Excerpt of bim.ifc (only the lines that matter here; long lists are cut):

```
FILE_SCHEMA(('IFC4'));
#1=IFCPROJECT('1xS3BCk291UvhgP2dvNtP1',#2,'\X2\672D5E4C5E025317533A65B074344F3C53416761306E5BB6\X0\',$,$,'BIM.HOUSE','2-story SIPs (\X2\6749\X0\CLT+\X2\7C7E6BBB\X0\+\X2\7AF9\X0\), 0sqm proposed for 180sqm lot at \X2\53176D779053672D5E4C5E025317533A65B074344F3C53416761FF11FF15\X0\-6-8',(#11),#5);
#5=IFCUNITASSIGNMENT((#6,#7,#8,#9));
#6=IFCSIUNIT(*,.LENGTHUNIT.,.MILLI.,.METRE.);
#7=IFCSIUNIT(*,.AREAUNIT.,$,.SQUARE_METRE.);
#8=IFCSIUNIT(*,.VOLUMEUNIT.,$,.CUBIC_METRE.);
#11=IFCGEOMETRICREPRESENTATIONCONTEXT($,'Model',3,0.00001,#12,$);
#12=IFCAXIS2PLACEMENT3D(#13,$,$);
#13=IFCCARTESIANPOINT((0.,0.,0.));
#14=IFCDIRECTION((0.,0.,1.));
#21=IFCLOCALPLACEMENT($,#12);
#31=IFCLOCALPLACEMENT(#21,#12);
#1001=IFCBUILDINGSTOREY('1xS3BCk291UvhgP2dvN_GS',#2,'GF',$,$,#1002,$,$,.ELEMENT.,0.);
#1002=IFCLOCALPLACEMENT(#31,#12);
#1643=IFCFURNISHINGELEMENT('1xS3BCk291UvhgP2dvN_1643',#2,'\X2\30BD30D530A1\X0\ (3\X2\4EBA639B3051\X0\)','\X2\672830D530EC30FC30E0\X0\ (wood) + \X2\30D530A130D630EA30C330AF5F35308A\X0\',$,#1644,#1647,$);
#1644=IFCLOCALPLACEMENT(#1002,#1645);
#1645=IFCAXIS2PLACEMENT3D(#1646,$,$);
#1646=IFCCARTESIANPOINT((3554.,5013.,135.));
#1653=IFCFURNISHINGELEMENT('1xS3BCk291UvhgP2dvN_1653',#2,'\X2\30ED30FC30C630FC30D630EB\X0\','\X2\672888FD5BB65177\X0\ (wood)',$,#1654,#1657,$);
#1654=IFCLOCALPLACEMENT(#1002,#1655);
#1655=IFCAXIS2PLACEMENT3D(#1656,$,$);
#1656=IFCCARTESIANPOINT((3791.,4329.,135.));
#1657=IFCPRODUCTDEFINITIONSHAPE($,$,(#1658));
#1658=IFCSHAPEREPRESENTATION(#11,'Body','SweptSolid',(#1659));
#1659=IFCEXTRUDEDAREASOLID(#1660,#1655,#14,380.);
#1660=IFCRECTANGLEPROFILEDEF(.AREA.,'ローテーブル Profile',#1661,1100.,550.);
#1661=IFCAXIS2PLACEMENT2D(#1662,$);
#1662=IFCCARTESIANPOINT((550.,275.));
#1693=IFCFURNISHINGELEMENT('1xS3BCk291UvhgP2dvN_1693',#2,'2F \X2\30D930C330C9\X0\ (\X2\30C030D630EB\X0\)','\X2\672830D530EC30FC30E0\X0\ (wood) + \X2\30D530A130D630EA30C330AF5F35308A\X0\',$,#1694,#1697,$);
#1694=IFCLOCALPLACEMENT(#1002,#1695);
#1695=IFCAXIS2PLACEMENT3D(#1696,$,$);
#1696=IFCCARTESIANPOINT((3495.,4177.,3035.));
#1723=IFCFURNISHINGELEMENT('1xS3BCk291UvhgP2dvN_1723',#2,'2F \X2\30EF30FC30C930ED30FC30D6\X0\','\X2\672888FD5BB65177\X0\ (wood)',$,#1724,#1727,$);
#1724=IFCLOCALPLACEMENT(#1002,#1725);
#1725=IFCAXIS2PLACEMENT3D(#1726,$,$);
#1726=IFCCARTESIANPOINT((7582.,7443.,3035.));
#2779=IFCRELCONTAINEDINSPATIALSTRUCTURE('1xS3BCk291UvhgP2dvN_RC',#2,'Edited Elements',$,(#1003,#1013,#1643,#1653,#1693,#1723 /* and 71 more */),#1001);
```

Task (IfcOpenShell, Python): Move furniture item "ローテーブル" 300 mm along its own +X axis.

```python
import ifcopenshell
import ifcopenshell.api.geometry
import ifcopenshell.util.placement
import ifcopenshell.util.unit

model = ifcopenshell.open("bim.ifc")
unit_scale = ifcopenshell.util.unit.calculate_unit_scale(model)

item = model.by_id(1653)
matrix = ifcopenshell.util.placement.get_local_placement(item.ObjectPlacement)
matrix[:3, 3] += matrix[:3, 0] * 0.3 / unit_scale
ifcopenshell.api.geometry.edit_object_placement(model, product=item, matrix=matrix, is_si=False)

print(ifcopenshell.util.placement.get_local_placement(item.ObjectPlacement).round(3) + 0.0)

model.write("bim-out.ifc")
```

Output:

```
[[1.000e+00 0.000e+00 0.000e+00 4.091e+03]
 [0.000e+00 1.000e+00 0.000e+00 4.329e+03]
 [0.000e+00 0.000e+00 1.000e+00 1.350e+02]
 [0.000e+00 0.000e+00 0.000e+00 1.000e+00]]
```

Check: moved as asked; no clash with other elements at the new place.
